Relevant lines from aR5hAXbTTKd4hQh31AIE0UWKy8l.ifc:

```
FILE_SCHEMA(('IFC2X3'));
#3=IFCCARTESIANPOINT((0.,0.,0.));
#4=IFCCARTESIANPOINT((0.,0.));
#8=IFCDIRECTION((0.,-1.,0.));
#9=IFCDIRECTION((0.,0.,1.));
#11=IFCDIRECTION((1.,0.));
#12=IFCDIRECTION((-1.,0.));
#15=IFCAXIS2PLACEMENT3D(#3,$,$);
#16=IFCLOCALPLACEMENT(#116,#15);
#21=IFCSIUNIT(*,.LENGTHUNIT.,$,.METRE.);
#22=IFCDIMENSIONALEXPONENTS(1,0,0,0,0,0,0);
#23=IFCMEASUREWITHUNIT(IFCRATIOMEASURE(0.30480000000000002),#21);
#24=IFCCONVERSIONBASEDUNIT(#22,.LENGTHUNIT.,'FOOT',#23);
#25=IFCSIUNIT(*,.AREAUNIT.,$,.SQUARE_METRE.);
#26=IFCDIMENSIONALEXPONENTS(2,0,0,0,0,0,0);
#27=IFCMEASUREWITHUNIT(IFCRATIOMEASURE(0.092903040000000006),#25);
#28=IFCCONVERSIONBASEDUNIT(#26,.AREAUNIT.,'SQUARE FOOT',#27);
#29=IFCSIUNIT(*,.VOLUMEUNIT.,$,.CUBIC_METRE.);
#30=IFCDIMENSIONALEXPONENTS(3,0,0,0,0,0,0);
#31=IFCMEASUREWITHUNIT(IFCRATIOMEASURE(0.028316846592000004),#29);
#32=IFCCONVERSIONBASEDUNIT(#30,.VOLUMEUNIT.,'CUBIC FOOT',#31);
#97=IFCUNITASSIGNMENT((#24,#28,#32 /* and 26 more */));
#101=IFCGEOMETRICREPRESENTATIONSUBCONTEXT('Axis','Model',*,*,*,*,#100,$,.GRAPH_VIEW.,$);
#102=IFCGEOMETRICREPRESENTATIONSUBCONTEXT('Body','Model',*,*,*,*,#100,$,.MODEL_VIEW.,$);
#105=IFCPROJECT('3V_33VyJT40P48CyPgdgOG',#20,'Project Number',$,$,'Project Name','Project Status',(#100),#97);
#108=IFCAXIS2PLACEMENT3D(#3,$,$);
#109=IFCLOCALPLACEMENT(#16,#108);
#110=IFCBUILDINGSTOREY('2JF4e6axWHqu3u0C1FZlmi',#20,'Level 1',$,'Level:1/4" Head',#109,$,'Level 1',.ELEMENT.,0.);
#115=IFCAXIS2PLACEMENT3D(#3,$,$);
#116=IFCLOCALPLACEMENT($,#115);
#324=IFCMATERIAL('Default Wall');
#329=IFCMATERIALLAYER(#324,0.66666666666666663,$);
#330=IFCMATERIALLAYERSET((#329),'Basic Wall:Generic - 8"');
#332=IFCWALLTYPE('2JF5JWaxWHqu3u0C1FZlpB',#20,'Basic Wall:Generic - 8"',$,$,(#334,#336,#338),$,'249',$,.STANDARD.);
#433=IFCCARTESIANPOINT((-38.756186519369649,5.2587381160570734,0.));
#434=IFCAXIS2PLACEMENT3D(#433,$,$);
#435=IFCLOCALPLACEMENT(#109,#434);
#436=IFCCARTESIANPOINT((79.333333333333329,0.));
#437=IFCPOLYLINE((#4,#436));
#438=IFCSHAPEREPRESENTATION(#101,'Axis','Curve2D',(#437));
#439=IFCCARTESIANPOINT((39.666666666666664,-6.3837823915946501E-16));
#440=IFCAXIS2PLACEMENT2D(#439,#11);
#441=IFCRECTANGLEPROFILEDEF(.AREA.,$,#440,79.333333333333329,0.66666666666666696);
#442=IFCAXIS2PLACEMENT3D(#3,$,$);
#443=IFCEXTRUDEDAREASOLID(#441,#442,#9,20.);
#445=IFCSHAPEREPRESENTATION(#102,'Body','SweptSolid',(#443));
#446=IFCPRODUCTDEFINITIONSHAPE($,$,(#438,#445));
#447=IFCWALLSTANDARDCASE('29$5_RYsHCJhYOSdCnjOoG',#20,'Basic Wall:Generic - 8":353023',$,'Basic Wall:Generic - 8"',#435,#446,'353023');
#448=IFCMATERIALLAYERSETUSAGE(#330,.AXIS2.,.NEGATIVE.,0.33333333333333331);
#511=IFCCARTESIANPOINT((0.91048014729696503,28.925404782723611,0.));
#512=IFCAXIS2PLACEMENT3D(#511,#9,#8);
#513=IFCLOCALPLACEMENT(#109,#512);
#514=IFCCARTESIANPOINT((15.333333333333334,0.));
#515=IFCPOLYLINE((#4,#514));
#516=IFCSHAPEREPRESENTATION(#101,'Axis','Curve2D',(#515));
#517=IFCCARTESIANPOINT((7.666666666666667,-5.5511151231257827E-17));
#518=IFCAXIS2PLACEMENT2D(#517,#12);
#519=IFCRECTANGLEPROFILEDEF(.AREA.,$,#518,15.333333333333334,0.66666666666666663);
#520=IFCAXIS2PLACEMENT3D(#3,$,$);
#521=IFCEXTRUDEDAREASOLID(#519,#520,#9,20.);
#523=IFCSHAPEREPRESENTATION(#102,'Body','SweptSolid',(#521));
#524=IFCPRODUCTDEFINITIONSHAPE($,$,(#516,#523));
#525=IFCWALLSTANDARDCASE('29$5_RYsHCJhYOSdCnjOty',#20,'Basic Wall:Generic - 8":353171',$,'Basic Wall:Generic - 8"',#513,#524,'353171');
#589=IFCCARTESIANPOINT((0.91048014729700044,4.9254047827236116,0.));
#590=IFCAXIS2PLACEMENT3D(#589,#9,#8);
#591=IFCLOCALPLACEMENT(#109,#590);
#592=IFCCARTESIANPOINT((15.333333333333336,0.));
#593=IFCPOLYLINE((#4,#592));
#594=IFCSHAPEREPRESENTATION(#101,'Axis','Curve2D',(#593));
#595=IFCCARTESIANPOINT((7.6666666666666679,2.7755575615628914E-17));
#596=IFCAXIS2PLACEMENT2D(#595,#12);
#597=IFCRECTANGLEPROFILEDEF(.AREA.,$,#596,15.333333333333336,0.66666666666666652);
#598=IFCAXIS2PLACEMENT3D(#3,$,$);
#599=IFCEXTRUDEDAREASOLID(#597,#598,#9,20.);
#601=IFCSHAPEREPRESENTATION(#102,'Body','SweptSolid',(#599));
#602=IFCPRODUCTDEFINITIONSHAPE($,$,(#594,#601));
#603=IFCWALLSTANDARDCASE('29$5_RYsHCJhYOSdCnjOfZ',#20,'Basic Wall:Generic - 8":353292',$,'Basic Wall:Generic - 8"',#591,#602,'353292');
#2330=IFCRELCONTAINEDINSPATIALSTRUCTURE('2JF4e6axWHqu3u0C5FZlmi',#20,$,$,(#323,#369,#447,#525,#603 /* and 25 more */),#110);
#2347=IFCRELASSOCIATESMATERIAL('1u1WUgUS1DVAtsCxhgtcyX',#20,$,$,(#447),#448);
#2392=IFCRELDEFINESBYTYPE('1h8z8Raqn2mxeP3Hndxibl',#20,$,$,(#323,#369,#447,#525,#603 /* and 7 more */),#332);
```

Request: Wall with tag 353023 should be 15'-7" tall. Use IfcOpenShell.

```python
import ifcopenshell
import ifcopenshell.geom
import ifcopenshell.util.representation
import ifcopenshell.util.shape
import ifcopenshell.util.unit

model = ifcopenshell.open("aR5hAXbTTKd4hQh31AIE0UWKy8l.ifc")
unit_scale = ifcopenshell.util.unit.calculate_unit_scale(model)
settings = ifcopenshell.geom.settings()


def volume(element):
    """Net volume in cubic metres, openings subtracted."""
    shape = ifcopenshell.geom.create_shape(settings, element)
    return ifcopenshell.util.shape.get_volume(shape.geometry)


wall = model.by_id(447)
before = volume(wall)

body = ifcopenshell.util.representation.get_representation(wall, "Model", "Body")
solid = body.Items[0]
old_height = solid.Depth
solid.Depth = 187 * 0.0254 / unit_scale
after = volume(wall)

print(f"height {old_height:g} -> {solid.Depth:g}, volume {before:.3f} -> {after:.3f} m3")

model.write("aR5hAXbTTKd4hQh31AIE0UWKy8l_updated.ifc")
```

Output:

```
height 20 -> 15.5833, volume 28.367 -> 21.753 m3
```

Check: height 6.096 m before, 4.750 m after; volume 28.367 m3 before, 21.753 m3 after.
